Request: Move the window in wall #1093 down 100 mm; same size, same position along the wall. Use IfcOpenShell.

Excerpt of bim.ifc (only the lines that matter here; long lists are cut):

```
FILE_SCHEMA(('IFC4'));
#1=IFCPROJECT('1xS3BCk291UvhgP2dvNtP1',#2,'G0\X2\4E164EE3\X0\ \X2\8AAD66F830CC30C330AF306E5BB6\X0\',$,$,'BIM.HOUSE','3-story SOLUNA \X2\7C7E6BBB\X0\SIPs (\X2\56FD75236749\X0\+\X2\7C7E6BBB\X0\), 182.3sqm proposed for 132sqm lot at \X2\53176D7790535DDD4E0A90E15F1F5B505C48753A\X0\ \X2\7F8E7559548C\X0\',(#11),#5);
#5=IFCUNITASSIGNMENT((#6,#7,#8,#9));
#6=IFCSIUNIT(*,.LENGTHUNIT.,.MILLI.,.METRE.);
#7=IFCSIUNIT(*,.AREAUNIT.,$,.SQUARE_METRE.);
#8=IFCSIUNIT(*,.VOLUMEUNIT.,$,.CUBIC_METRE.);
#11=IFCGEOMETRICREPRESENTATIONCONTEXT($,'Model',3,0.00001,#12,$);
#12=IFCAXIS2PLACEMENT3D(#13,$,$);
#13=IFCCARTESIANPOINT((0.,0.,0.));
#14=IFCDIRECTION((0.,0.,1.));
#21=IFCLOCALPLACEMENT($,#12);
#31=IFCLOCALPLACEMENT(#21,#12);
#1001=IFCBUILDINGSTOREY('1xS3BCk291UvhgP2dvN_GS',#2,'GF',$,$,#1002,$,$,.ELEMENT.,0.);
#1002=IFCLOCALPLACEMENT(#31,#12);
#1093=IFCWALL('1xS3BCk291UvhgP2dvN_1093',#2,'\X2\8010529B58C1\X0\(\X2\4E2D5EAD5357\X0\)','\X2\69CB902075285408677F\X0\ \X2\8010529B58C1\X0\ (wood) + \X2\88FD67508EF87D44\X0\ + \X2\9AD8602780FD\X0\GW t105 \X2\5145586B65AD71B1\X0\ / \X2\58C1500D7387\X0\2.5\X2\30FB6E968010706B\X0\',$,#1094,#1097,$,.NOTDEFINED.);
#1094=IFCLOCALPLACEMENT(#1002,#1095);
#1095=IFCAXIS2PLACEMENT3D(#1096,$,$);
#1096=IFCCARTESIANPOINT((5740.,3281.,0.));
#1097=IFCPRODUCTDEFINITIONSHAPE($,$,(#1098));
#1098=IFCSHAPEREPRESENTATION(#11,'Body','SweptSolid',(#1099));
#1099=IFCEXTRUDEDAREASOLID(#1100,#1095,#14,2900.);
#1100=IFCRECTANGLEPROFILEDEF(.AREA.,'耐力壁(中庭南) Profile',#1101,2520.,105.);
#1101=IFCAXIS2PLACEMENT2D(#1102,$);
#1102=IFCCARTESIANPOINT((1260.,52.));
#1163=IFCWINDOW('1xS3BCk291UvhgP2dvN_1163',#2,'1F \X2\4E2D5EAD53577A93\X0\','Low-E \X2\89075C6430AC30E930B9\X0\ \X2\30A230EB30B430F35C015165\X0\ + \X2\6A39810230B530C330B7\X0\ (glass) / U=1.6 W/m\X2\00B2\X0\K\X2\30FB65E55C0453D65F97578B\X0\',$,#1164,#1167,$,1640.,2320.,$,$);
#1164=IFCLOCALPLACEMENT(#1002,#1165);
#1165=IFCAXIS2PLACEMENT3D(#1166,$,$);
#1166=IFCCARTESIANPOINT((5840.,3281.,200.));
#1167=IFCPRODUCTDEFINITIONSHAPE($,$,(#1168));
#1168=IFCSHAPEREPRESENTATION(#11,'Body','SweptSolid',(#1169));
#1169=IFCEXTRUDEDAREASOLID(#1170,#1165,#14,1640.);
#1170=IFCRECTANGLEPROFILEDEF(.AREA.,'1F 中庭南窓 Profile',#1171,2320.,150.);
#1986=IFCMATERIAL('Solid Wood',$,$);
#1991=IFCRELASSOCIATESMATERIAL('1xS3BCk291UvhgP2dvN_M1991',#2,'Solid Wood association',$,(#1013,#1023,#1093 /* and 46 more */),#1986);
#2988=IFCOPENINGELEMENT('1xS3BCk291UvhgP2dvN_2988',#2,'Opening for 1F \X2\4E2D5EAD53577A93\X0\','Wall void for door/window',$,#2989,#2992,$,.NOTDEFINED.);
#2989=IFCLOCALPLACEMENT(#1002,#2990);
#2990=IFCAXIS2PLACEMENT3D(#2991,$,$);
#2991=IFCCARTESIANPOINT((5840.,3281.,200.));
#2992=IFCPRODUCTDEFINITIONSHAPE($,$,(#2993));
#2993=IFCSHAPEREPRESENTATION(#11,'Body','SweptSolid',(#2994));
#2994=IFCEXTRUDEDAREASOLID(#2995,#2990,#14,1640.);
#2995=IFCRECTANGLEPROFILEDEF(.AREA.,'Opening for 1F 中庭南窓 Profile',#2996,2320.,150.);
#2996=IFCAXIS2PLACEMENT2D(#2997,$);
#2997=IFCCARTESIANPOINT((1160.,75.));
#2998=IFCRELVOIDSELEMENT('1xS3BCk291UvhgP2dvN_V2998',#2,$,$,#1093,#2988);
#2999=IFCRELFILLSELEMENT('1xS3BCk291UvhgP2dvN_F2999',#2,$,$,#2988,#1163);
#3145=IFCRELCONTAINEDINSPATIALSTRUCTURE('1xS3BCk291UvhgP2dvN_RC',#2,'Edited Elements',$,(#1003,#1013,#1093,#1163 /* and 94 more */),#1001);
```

```python
import numpy as np
import ifcopenshell
import ifcopenshell.api.geometry
import ifcopenshell.util.placement
import ifcopenshell.util.unit

model = ifcopenshell.open("bim.ifc")
unit_scale = ifcopenshell.util.unit.calculate_unit_scale(model)

window = model.by_guid("1xS3BCk291UvhgP2dvN_1163")
opening = window.FillsVoids[0].RelatingOpeningElement
dz = -0.1 / unit_scale

shift = np.array([0.0, 0.0, dz])
# The window is not placed relative to its opening, so move both.
for product in (opening, window):
    matrix = ifcopenshell.util.placement.get_local_placement(product.ObjectPlacement)
    matrix[:3, 3] += shift
    ifcopenshell.api.geometry.edit_object_placement(model, product=product, matrix=matrix, is_si=False)

print(f"moved by {dz * unit_scale:+.3f} m")

model.write("bim_updated.ifc")
```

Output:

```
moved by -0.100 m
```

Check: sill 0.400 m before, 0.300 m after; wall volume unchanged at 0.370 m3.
